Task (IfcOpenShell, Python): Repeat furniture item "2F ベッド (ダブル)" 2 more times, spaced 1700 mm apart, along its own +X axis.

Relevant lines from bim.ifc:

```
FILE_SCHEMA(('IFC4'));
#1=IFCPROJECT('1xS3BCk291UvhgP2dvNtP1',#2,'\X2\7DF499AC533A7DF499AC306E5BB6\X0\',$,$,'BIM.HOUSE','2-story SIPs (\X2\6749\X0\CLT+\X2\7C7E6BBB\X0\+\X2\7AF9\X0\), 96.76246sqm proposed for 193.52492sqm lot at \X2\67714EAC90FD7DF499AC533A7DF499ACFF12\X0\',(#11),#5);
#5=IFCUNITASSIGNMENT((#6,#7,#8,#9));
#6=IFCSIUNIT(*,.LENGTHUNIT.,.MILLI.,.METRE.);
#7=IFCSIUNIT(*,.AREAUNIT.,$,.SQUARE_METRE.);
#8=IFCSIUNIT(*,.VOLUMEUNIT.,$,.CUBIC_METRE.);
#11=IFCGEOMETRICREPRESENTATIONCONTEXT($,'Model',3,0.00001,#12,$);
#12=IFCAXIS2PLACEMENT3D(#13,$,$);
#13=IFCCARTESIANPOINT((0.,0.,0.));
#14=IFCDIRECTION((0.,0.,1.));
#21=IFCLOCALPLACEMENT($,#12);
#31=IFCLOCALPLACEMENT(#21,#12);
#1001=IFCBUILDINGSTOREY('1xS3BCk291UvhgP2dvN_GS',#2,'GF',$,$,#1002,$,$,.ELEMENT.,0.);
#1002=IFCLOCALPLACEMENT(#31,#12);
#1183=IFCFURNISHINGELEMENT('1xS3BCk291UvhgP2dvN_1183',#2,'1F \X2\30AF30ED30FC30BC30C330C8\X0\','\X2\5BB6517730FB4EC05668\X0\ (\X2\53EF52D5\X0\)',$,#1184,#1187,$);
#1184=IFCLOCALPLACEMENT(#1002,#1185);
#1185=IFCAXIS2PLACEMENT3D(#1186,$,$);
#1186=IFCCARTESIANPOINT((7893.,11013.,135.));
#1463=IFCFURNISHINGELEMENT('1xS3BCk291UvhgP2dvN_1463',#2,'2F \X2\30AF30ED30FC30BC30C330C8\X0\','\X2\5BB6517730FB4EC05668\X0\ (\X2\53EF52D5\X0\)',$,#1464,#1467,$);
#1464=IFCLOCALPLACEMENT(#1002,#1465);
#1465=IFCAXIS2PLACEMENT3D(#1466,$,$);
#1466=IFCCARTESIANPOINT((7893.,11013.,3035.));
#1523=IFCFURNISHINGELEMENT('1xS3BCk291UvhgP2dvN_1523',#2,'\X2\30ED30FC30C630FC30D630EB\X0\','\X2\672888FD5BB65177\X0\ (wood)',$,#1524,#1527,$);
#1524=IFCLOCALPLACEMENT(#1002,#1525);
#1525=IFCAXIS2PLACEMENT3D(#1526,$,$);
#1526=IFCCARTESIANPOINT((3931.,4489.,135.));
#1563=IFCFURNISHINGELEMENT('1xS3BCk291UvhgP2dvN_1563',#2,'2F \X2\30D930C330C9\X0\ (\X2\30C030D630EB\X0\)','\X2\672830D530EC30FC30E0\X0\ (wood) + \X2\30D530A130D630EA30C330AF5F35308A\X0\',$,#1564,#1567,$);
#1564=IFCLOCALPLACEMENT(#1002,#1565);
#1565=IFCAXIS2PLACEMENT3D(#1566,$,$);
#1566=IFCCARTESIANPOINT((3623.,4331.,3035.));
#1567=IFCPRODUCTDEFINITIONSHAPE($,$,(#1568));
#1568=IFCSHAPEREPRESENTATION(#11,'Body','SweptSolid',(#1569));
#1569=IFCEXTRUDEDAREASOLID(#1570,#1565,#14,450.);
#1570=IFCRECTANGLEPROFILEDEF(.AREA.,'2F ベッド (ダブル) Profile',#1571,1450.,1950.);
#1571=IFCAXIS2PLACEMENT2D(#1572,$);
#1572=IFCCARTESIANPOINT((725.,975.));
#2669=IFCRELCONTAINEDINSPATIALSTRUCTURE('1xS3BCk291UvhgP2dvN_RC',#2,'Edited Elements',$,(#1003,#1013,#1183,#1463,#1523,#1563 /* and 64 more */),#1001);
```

```python
import ifcopenshell
import ifcopenshell.api.geometry
import ifcopenshell.api.root
import ifcopenshell.util.element
import ifcopenshell.util.placement
import ifcopenshell.util.unit

model = ifcopenshell.open("bim.ifc")
unit_scale = ifcopenshell.util.unit.calculate_unit_scale(model)


def reuse_history(source, copy):
    """copy_class also copies each property set's owner history, people and application; keep the originals."""
    for rel in copy.IsDefinedBy:
        if rel.is_a("IfcRelDefinesByProperties") and (history := rel.RelatingPropertyDefinition.OwnerHistory):
            rel.RelatingPropertyDefinition.OwnerHistory = source.OwnerHistory
            ifcopenshell.util.element.remove_deep2(model, history)


source = model.by_guid("1xS3BCk291UvhgP2dvN_1563")
base = ifcopenshell.util.placement.get_local_placement(source.ObjectPlacement)
step = base[:3, 0] * 1.7 / unit_scale

for i in range(1, 3):
    copy = ifcopenshell.api.root.copy_class(model, product=source)
    copy.Representation = ifcopenshell.util.element.copy_deep(
        model, source.Representation, exclude=["IfcGeometricRepresentationContext", "IfcRepresentationMap"]
    )
    reuse_history(source, copy)
    matrix = base.copy()
    matrix[:3, 3] += i * step
    print("added at", matrix[:3, 3].round(3) + 0.0)
    ifcopenshell.api.geometry.edit_object_placement(model, product=copy, matrix=matrix, is_si=False)

model.write("bim_updated.ifc")
```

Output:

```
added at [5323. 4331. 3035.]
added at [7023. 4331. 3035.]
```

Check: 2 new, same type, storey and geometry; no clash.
